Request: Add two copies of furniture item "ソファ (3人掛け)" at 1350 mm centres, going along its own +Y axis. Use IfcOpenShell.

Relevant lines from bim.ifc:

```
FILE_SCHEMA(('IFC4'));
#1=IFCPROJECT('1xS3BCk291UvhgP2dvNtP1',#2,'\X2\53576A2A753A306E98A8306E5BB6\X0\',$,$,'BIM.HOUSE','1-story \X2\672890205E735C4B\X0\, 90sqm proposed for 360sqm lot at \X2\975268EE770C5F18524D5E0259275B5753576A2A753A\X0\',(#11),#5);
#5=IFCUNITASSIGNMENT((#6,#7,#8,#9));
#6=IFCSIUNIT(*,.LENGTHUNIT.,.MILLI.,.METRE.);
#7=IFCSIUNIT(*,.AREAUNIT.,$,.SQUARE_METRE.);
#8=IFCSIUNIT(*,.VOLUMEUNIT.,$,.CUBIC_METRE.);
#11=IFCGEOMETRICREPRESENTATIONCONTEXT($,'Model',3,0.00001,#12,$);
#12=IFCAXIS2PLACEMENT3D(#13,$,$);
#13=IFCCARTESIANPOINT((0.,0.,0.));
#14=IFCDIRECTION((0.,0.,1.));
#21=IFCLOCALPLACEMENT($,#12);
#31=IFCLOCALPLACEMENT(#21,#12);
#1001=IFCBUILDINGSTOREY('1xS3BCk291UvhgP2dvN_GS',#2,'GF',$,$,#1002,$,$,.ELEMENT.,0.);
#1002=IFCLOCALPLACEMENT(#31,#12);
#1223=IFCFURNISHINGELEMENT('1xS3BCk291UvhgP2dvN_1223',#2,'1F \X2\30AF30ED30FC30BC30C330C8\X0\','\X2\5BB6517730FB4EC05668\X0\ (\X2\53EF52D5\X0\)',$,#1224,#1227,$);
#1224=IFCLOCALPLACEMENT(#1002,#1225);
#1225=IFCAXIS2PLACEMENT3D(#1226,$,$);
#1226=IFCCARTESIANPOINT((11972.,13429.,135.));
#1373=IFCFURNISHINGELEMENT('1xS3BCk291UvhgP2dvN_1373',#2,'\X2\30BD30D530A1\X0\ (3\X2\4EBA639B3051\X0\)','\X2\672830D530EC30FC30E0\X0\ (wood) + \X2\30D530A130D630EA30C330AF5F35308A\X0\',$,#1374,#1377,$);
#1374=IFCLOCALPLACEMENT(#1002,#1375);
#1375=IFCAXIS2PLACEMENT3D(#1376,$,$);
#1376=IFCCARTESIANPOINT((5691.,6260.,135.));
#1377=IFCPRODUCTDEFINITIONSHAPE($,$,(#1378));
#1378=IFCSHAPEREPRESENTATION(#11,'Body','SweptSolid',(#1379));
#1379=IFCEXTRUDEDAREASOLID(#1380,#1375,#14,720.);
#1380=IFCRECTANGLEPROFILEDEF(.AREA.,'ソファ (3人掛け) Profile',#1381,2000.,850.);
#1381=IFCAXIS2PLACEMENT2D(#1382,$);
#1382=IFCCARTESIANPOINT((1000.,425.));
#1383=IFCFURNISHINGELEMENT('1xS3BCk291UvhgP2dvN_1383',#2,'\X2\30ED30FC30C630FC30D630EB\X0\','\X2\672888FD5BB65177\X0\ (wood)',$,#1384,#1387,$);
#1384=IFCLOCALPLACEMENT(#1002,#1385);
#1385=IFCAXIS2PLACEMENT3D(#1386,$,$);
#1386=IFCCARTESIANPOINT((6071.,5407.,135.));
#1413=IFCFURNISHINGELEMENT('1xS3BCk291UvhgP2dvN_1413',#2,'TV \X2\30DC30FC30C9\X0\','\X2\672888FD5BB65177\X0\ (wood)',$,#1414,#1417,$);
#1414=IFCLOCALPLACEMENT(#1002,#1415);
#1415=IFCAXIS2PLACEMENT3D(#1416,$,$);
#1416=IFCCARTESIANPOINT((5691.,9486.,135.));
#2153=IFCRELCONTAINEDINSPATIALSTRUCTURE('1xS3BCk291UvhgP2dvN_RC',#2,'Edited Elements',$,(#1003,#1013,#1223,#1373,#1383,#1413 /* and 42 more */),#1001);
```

```python
import ifcopenshell
import ifcopenshell.api.geometry
import ifcopenshell.api.root
import ifcopenshell.util.element
import ifcopenshell.util.placement

model = ifcopenshell.open("bim.ifc")


def reuse_history(source, copy):
    """copy_class also copies each property set's owner history, people and application; keep the originals."""
    for rel in copy.IsDefinedBy:
        if rel.is_a("IfcRelDefinesByProperties") and (history := rel.RelatingPropertyDefinition.OwnerHistory):
            rel.RelatingPropertyDefinition.OwnerHistory = source.OwnerHistory
            ifcopenshell.util.element.remove_deep2(model, history)


source = model.by_guid("1xS3BCk291UvhgP2dvN_1373")
base = ifcopenshell.util.placement.get_local_placement(source.ObjectPlacement)
step = base[:3, 1] * 1350.0

for i in range(1, 3):
    copy = ifcopenshell.api.root.copy_class(model, product=source)
    copy.Representation = ifcopenshell.util.element.copy_deep(
        model, source.Representation, exclude=["IfcGeometricRepresentationContext", "IfcRepresentationMap"]
    )
    reuse_history(source, copy)
    matrix = base.copy()
    matrix[:3, 3] += i * step
    print("added at", matrix[:3, 3].round(3) + 0.0)
    ifcopenshell.api.geometry.edit_object_placement(model, product=copy, matrix=matrix, is_si=False)

model.write("bim_v2.ifc")
```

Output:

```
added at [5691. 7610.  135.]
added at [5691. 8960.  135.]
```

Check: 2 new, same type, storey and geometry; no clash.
